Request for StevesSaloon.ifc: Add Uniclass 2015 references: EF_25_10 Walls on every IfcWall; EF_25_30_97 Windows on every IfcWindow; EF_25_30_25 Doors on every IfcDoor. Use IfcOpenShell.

First a look at what the model holds.

```python
import ifcopenshell

model = ifcopenshell.open("StevesSaloon.ifc")
print(model.schema)
print("classifications:", [c.Name for c in model.by_type("IfcClassification")])
for ifc_class in ("IfcDoor", "IfcRoof", "IfcStair", "IfcWall", "IfcWindow"):
    print(ifc_class, len(model.by_type(ifc_class)))
```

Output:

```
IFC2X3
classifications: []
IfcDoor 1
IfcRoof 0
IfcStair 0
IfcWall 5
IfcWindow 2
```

```python
import ifcopenshell
import ifcopenshell.api.classification

model = ifcopenshell.open("StevesSaloon.ifc")

# IFC2X3 requires Source and Edition and has no link from the project to the system.
system = model.create_entity("IfcClassification", Source="NBS", Edition="2015", Name="Uniclass 2015")

codes = {
    "IfcWall": ("EF_25_10", "Walls"),
    "IfcWindow": ("EF_25_30_97", "Windows"),
    "IfcDoor": ("EF_25_30_25", "Doors"),
}
for ifc_class, (code, name) in codes.items():
    products = model.by_type(ifc_class)
    ifcopenshell.api.classification.add_reference(
        model, products=products, classification=system, identification=code, name=name
    )
    print(code, len(products))

model.write("StevesSaloon_rev.ifc")
```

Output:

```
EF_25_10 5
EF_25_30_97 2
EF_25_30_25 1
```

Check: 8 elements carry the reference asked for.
